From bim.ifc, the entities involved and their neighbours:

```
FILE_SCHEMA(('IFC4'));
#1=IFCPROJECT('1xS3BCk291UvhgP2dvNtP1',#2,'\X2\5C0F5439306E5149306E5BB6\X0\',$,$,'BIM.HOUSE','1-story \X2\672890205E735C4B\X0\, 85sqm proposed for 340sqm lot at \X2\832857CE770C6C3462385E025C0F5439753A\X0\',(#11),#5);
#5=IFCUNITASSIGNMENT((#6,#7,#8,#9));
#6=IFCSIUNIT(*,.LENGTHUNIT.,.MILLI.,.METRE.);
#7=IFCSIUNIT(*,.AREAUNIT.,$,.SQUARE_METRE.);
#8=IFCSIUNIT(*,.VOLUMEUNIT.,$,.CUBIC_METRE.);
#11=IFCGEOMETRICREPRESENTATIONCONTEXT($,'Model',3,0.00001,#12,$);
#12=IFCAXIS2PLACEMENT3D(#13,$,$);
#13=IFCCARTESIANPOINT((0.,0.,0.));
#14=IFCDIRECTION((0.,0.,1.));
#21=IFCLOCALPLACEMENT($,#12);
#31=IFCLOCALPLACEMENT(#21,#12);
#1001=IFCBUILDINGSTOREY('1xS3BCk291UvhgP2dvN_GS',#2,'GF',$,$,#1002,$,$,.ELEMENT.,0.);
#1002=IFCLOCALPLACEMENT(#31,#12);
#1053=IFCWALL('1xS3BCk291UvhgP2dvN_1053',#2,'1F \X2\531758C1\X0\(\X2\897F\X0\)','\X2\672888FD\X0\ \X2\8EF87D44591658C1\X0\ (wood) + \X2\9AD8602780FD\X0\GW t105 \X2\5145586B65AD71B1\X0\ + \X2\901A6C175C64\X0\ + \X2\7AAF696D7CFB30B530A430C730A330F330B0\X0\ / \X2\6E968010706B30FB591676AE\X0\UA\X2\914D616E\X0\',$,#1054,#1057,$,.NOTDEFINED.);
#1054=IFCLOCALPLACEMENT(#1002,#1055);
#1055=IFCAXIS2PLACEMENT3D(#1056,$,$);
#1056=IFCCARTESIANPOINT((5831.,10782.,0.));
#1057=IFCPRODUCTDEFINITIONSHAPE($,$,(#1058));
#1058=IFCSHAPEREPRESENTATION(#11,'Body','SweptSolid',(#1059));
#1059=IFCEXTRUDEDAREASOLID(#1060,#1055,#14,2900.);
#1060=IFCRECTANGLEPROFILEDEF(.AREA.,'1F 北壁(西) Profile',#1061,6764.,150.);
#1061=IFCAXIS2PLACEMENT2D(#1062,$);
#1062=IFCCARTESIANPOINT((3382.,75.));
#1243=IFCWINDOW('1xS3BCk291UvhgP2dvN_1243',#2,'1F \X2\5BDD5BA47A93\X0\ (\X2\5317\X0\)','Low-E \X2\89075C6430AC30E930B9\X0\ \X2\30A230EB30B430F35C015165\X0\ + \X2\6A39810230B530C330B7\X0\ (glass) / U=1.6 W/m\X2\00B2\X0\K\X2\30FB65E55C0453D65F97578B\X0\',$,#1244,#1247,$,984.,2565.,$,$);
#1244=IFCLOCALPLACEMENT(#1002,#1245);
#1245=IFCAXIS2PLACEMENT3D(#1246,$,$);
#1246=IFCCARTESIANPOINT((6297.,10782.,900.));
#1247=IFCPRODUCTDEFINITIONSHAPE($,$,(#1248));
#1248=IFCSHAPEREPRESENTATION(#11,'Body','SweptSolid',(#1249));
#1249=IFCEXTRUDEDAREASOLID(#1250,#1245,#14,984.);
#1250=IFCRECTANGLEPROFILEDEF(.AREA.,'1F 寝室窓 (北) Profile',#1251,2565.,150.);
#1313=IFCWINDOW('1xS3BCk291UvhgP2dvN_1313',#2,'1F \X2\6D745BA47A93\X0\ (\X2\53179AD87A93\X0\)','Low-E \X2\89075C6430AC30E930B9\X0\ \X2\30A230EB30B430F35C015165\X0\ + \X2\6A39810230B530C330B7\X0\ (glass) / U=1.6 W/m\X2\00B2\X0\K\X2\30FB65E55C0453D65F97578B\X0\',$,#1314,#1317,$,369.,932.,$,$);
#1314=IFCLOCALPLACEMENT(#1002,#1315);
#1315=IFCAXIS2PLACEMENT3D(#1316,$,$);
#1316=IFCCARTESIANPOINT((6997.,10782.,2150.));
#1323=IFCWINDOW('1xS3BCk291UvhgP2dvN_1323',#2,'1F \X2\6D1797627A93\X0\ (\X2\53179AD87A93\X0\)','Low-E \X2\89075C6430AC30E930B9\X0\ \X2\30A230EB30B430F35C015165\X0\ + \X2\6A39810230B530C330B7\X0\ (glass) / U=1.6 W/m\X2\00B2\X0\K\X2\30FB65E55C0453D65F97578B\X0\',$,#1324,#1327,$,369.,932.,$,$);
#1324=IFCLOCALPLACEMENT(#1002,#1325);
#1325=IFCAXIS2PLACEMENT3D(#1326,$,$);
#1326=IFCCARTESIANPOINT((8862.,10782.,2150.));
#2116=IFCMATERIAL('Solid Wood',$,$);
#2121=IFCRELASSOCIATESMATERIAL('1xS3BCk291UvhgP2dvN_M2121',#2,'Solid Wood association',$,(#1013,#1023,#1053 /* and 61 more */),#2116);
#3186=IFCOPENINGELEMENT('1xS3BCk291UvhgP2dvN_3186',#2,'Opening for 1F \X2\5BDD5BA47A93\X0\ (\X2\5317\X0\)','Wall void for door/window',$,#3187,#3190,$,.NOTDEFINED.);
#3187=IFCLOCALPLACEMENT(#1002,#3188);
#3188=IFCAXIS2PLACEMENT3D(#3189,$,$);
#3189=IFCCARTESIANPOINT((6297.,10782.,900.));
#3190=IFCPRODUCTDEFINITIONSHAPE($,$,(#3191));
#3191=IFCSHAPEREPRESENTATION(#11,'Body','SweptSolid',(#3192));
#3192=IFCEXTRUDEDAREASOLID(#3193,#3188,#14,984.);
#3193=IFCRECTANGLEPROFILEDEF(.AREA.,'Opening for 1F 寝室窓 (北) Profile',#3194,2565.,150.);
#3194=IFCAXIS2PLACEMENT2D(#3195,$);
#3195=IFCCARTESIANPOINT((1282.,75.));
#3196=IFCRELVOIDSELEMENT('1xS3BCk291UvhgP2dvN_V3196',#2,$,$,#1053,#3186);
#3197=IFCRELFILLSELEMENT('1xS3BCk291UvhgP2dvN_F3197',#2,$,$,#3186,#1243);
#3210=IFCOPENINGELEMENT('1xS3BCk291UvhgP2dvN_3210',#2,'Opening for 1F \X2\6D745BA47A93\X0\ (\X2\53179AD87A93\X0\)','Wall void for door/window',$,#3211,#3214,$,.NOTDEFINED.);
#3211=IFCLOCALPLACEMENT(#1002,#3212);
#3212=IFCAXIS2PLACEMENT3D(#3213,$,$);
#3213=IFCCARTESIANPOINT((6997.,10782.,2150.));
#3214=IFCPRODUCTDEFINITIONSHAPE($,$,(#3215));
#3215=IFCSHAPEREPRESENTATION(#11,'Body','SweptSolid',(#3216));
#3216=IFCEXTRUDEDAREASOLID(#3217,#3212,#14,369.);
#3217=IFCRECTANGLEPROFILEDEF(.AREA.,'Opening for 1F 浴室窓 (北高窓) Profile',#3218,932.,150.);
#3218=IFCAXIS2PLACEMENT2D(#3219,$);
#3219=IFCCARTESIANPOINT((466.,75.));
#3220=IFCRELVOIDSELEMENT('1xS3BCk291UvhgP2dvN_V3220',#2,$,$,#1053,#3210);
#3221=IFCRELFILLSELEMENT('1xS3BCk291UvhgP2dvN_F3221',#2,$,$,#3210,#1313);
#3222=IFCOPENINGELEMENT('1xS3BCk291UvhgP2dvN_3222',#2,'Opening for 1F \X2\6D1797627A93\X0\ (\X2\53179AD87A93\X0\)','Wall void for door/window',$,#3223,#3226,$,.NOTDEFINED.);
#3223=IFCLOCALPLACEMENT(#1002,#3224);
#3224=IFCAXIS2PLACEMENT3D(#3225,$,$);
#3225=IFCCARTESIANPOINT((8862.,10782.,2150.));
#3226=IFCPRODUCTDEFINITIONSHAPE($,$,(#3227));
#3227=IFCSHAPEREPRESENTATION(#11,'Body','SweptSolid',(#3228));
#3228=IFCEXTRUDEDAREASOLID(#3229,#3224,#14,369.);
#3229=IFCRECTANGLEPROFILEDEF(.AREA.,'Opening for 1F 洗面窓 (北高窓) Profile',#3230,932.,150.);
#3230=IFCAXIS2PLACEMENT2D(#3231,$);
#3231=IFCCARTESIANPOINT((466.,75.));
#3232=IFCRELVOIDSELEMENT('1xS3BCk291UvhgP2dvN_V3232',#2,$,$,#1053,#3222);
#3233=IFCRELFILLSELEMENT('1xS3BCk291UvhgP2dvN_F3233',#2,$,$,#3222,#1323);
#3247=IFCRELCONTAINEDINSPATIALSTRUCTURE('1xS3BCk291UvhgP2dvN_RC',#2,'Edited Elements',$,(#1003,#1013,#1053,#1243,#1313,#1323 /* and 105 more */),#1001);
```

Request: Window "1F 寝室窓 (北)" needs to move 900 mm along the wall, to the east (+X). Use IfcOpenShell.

```python
import ifcopenshell
import ifcopenshell.api.geometry
import ifcopenshell.util.placement
import ifcopenshell.util.unit

model = ifcopenshell.open("bim.ifc")
unit_scale = ifcopenshell.util.unit.calculate_unit_scale(model)

window = model.by_guid("1xS3BCk291UvhgP2dvN_1243")
opening = window.FillsVoids[0].RelatingOpeningElement
wall = opening.VoidsElements[0].RelatingBuildingElement

wall_matrix = ifcopenshell.util.placement.get_local_placement(wall.ObjectPlacement)
shift = wall_matrix[:3, 0] * 0.9 / unit_scale
before = ifcopenshell.util.placement.get_local_placement(window.ObjectPlacement)[:3, 3].copy()

# The window is not placed relative to its opening, so move both.
for product in (opening, window):
    matrix = ifcopenshell.util.placement.get_local_placement(product.ObjectPlacement)
    matrix[:3, 3] += shift
    ifcopenshell.api.geometry.edit_object_placement(model, product=product, matrix=matrix, is_si=False)

after = ifcopenshell.util.placement.get_local_placement(window.ObjectPlacement)[:3, 3]
print("window moved by", (after - before).round(3) + 0.0)

model.write("bim_edited.ifc")
```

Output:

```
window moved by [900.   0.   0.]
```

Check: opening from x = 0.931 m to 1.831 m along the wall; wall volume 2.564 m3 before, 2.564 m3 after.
